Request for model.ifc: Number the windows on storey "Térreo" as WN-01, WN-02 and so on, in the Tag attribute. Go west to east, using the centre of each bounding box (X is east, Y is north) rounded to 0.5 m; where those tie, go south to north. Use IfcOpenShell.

First a look at what the model holds.

```python
import ifcopenshell
import ifcopenshell.util.element
import ifcopenshell.util.placement

model = ifcopenshell.open("model.ifc")
print(model.schema)
storey = next(s for s in model.by_type("IfcBuildingStorey") if s.Name == "Térreo")
windows = [e for e in ifcopenshell.util.element.get_decomposition(storey) if e.is_a("IfcWindow")]
for e in sorted(windows, key=lambda e: e.id()):
    origin = ifcopenshell.util.placement.get_local_placement(e.ObjectPlacement)[:3, 3]
    print(e.id(), e.Tag, e.Name, origin.round(2) + 0.0, sep=" | ")
```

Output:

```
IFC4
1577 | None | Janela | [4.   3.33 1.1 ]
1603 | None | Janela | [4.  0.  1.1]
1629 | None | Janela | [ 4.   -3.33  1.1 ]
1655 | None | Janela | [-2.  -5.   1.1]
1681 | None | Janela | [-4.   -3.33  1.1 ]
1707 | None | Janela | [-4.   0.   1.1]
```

```python
import ifcopenshell
import ifcopenshell.geom
import ifcopenshell.util.element
import ifcopenshell.util.shape

model = ifcopenshell.open("model.ifc")
settings = ifcopenshell.geom.settings()
settings.set("use-world-coords", True)


def centre(element):
    shape = ifcopenshell.geom.create_shape(settings, element)
    return ifcopenshell.util.shape.get_bbox_centroid(shape.geometry)


storey = next(s for s in model.by_type("IfcBuildingStorey") if s.Name == "Térreo")
windows = [e for e in ifcopenshell.util.element.get_decomposition(storey) if e.is_a("IfcWindow")]

# Insertion points can sit at a corner or the storey origin, so sort by the geometry (in metres).
centres = {e: centre(e) for e in windows}
windows.sort(key=lambda e: (round(centres[e][0] / 0.5), centres[e][1]))

for i, e in enumerate(windows, start=1):
    number = f"WN-{i:02d}"
    e.Tag = number
    print(e.id(), number)

model.write("model_rev.ifc")
```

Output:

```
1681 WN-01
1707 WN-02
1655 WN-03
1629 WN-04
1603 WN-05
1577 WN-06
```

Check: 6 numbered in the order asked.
